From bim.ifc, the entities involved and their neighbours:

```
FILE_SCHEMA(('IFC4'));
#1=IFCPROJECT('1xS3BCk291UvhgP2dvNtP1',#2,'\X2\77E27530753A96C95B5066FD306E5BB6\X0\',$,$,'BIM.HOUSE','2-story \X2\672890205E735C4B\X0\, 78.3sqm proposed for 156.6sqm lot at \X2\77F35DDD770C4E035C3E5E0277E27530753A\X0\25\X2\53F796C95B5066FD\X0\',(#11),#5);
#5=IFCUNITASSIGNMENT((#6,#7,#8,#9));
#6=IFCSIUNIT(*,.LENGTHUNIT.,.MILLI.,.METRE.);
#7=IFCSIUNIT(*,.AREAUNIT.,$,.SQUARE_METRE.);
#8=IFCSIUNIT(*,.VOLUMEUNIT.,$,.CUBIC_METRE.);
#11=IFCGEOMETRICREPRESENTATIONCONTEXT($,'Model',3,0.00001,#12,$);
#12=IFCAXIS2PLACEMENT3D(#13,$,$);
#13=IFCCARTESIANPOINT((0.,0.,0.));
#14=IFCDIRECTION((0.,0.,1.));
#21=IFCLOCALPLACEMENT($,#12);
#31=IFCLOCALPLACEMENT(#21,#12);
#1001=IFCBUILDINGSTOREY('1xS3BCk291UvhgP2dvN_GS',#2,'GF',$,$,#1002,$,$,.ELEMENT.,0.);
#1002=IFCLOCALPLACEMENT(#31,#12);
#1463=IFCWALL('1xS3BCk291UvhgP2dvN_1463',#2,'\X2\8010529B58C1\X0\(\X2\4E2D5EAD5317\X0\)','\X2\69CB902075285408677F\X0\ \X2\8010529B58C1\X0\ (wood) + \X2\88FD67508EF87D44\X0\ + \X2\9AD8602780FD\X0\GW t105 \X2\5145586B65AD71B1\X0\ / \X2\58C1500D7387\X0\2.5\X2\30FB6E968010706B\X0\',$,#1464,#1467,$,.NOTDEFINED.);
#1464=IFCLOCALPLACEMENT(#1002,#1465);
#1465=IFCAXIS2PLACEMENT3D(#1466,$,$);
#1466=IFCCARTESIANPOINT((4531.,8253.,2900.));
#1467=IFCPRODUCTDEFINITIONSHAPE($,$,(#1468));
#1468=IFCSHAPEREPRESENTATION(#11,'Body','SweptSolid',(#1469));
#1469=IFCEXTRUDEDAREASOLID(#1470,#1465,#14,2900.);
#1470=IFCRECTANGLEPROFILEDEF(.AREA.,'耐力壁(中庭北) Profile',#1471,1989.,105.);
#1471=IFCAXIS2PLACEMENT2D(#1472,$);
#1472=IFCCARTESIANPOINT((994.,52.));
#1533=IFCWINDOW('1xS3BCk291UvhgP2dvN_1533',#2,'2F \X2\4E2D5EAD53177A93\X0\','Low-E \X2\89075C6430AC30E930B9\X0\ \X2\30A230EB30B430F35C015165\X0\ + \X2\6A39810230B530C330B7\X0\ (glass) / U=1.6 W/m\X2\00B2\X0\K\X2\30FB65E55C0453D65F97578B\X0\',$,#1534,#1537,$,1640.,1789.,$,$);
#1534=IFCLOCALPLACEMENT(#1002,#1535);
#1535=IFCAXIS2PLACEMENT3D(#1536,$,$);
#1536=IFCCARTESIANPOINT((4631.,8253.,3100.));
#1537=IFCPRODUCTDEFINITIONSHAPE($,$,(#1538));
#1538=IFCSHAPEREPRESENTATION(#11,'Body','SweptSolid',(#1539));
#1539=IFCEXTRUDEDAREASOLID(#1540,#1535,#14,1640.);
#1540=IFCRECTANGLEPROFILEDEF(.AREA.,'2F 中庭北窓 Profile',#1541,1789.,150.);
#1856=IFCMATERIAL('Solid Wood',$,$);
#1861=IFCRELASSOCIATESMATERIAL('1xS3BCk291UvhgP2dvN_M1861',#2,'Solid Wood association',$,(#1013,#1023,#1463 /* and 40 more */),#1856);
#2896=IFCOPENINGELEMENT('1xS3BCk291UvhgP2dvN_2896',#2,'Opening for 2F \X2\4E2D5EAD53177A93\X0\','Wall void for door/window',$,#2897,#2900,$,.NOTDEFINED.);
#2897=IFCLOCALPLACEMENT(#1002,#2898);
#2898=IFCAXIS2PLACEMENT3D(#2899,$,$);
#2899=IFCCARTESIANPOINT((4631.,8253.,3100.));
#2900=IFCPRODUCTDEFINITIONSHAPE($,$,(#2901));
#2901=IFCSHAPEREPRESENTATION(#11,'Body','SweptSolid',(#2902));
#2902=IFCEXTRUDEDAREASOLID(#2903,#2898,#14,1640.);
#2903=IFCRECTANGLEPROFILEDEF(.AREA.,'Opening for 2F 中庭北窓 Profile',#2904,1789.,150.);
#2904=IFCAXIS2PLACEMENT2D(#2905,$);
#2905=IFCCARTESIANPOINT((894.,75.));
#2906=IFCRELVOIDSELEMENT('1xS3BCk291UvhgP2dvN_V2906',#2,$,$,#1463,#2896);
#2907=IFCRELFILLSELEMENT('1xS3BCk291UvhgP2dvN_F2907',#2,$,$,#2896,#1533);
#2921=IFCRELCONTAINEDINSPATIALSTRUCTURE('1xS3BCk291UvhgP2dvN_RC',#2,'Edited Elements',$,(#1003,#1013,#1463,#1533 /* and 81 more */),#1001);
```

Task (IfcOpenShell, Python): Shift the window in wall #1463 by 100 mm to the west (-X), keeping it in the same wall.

```python
import ifcopenshell
import ifcopenshell.api.geometry
import ifcopenshell.util.placement
import ifcopenshell.util.unit

model = ifcopenshell.open("bim.ifc")
unit_scale = ifcopenshell.util.unit.calculate_unit_scale(model)

window = model.by_id(1533)
opening = window.FillsVoids[0].RelatingOpeningElement
wall = opening.VoidsElements[0].RelatingBuildingElement

wall_matrix = ifcopenshell.util.placement.get_local_placement(wall.ObjectPlacement)
shift = wall_matrix[:3, 0] * -0.1 / unit_scale
before = ifcopenshell.util.placement.get_local_placement(window.ObjectPlacement)[:3, 3].copy()

# The window is not placed relative to its opening, so move both.
for product in (opening, window):
    matrix = ifcopenshell.util.placement.get_local_placement(product.ObjectPlacement)
    matrix[:3, 3] += shift
    ifcopenshell.api.geometry.edit_object_placement(model, product=product, matrix=matrix, is_si=False)

after = ifcopenshell.util.placement.get_local_placement(window.ObjectPlacement)[:3, 3]
print("window moved by", (after - before).round(3) + 0.0)

model.write("bim_updated.ifc")
```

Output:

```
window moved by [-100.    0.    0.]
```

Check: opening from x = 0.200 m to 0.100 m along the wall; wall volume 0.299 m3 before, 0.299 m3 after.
